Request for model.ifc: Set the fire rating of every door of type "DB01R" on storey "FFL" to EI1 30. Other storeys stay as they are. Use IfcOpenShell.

First a look at what the model holds.

```python
import ifcopenshell
import ifcopenshell.util.element

model = ifcopenshell.open("model.ifc")
print(model.schema)
storey = next(s for s in model.by_type("IfcBuildingStorey") if s.Name == "FFL")
doors = [e for e in ifcopenshell.util.element.get_decomposition(storey) if e.is_a("IfcDoor")]
seen = {}
for e in doors:
    element_type = ifcopenshell.util.element.get_type(e)
    key = (element_type.Name if element_type != e and element_type else None, ifcopenshell.util.element.get_pset(e, "Pset_DoorCommon", "FireRating"))
    seen[key] = seen.get(key, 0) + 1
for (name, value), count in sorted(seen.items(), key=str):
    print(count, "x", name, "|", value)
```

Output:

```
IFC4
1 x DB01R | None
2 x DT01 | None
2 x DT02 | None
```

```python
import ifcopenshell
import ifcopenshell.api.pset
import ifcopenshell.util.element

model = ifcopenshell.open("model.ifc")

storey = next(s for s in model.by_type("IfcBuildingStorey") if s.Name == "FFL")
doors = [e for e in ifcopenshell.util.element.get_decomposition(storey) if e.is_a("IfcDoor")]

count = 0
for e in doors:
    element_type = ifcopenshell.util.element.get_type(e)
    if element_type in (None, e) or element_type.Name != "DB01R":
        continue
    # add_pset returns the element's existing set when there is one.
    pset = ifcopenshell.api.pset.add_pset(model, product=e, name="Pset_DoorCommon")
    ifcopenshell.api.pset.edit_pset(model, pset=pset, properties={"FireRating": "EI1 30"})
    count += 1

print(count, "doors updated")

model.write("model_edited.ifc")
```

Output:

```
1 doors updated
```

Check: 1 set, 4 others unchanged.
